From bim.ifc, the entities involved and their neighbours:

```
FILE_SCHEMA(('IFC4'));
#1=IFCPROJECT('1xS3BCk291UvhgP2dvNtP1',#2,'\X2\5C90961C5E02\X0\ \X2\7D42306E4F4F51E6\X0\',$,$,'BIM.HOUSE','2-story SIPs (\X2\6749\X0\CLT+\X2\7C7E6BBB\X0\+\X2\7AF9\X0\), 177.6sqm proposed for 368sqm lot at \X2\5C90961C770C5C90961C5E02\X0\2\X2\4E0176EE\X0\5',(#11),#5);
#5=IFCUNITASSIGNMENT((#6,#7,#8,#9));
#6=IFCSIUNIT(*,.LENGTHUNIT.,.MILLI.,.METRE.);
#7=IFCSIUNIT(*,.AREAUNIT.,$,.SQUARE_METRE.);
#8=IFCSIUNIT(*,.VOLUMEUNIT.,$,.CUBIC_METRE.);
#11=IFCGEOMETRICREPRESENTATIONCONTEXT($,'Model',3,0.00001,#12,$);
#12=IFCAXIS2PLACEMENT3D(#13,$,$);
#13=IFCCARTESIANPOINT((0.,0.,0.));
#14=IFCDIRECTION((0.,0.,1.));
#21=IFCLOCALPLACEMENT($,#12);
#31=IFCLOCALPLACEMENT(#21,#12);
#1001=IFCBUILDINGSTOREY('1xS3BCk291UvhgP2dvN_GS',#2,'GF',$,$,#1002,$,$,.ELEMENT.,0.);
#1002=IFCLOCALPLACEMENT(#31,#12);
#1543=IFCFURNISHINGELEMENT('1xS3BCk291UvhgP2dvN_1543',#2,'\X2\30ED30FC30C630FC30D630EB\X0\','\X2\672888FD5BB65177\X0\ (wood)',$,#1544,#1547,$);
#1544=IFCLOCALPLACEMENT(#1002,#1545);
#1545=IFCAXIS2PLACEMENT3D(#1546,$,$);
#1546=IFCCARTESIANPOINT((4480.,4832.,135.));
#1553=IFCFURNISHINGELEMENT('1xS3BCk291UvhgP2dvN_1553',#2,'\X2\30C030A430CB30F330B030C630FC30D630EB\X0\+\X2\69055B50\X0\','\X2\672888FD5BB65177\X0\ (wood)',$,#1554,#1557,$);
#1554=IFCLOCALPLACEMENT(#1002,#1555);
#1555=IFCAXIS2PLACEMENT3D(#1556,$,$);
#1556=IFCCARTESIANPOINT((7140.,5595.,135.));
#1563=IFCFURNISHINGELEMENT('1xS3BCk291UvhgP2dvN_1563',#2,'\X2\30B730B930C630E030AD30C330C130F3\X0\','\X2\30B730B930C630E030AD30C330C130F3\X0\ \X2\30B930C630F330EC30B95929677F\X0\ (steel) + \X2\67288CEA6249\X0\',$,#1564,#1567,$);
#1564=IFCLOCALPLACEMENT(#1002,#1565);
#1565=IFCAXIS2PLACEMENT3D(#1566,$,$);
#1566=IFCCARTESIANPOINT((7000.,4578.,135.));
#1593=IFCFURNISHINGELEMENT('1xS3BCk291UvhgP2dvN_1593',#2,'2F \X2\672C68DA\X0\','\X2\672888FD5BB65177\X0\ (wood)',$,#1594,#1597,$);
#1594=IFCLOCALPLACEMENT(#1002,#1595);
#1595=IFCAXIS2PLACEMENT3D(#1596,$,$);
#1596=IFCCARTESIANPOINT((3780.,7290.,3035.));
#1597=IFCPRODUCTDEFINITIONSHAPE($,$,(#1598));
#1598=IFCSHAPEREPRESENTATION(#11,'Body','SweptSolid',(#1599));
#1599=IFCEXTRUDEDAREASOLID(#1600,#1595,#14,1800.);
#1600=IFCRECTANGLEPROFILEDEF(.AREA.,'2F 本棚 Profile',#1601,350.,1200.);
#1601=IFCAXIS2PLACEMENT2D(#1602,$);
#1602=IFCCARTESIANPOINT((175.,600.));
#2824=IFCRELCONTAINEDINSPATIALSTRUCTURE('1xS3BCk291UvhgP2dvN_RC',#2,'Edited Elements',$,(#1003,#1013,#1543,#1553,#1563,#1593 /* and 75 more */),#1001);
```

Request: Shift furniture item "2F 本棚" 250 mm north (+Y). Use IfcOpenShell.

```python
import ifcopenshell
import ifcopenshell.api.geometry
import ifcopenshell.util.placement
import ifcopenshell.util.unit

model = ifcopenshell.open("bim.ifc")
unit_scale = ifcopenshell.util.unit.calculate_unit_scale(model)

item = model.by_guid("1xS3BCk291UvhgP2dvN_1593")
matrix = ifcopenshell.util.placement.get_local_placement(item.ObjectPlacement)
matrix[1, 3] += 0.25 / unit_scale
ifcopenshell.api.geometry.edit_object_placement(model, product=item, matrix=matrix, is_si=False)

print(ifcopenshell.util.placement.get_local_placement(item.ObjectPlacement).round(3) + 0.0)

model.write("bim_v2.ifc")
```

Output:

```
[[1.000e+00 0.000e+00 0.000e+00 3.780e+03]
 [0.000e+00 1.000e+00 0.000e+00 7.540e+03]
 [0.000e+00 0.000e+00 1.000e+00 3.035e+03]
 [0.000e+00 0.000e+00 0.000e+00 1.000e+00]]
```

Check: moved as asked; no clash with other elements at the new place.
